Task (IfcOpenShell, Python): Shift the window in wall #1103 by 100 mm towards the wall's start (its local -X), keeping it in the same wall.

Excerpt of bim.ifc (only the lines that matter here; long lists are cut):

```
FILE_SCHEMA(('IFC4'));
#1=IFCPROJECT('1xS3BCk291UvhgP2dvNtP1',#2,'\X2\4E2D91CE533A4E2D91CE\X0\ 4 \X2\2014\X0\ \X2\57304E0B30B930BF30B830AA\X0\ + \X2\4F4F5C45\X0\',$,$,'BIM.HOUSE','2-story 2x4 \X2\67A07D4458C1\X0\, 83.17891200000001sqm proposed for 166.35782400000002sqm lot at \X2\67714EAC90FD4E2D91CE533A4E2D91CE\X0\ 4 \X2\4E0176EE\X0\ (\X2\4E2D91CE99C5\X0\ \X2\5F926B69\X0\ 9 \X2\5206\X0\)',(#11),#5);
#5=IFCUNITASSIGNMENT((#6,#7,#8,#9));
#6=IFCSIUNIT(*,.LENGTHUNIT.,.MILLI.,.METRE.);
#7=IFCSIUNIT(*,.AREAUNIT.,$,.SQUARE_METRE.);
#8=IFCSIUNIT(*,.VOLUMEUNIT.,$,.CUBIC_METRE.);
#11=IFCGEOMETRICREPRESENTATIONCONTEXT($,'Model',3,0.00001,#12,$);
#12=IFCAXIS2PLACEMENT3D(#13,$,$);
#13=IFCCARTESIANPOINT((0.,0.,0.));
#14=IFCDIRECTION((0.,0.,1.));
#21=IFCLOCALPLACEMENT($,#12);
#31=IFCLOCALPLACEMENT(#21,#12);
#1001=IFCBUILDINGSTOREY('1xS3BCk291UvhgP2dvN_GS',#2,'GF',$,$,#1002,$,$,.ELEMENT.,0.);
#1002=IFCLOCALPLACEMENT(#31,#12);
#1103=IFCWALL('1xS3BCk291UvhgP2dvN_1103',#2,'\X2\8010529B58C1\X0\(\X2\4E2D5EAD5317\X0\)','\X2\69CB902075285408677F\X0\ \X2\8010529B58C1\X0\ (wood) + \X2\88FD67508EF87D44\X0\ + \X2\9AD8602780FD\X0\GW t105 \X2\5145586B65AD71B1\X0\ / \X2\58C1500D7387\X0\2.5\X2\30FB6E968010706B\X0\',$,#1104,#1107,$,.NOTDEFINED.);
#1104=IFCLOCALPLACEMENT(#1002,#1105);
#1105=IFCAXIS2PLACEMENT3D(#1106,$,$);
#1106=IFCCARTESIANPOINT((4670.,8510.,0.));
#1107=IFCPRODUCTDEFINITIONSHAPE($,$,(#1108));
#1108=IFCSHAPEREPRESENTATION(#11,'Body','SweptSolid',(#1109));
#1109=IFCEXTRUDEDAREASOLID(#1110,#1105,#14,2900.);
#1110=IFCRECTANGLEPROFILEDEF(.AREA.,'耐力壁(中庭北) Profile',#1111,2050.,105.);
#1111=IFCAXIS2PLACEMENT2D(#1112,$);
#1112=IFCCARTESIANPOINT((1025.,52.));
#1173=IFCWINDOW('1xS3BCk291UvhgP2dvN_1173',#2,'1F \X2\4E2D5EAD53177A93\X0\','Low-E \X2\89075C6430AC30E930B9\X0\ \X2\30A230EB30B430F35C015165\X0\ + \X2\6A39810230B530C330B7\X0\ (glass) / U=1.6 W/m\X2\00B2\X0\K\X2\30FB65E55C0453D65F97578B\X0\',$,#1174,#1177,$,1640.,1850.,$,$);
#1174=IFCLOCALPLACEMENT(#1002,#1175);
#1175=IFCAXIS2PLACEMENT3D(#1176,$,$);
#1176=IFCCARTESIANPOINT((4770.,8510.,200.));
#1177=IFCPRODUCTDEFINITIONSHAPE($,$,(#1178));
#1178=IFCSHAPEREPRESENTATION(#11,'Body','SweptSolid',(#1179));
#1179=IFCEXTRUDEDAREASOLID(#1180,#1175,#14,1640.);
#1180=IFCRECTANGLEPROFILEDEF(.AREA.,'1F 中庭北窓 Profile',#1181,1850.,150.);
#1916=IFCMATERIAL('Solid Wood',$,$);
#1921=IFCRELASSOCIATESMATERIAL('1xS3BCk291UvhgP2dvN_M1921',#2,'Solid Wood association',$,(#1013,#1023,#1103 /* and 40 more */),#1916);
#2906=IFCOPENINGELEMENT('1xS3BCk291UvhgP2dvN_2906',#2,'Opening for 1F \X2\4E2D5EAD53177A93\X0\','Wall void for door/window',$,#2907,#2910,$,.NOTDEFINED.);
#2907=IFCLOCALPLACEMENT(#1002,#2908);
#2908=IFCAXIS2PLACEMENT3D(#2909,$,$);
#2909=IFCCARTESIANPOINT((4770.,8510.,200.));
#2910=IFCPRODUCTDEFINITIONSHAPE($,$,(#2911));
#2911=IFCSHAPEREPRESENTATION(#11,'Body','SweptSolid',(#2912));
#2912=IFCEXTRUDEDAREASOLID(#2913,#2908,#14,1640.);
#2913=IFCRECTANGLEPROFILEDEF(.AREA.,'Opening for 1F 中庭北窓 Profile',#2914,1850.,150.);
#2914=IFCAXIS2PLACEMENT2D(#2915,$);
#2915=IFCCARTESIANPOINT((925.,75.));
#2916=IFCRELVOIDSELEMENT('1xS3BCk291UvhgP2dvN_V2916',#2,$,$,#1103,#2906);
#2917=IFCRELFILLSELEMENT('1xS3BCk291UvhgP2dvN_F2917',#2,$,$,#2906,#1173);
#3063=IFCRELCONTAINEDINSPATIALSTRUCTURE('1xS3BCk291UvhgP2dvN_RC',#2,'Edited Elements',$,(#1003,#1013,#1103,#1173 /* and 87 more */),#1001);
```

```python
import ifcopenshell
import ifcopenshell.api.geometry
import ifcopenshell.util.placement
import ifcopenshell.util.unit

model = ifcopenshell.open("bim.ifc")
unit_scale = ifcopenshell.util.unit.calculate_unit_scale(model)

window = model.by_guid("1xS3BCk291UvhgP2dvN_1173")
opening = window.FillsVoids[0].RelatingOpeningElement
wall = opening.VoidsElements[0].RelatingBuildingElement

wall_matrix = ifcopenshell.util.placement.get_local_placement(wall.ObjectPlacement)
shift = wall_matrix[:3, 0] * -0.1 / unit_scale
before = ifcopenshell.util.placement.get_local_placement(window.ObjectPlacement)[:3, 3].copy()

# The window is not placed relative to its opening, so move both.
for product in (opening, window):
    matrix = ifcopenshell.util.placement.get_local_placement(product.ObjectPlacement)
    matrix[:3, 3] += shift
    ifcopenshell.api.geometry.edit_object_placement(model, product=product, matrix=matrix, is_si=False)

after = ifcopenshell.util.placement.get_local_placement(window.ObjectPlacement)[:3, 3]
print("window moved by", (after - before).round(3) + 0.0)

model.write("bim_updated.ifc")
```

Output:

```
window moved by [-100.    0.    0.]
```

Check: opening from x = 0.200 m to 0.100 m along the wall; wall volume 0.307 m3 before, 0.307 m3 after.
